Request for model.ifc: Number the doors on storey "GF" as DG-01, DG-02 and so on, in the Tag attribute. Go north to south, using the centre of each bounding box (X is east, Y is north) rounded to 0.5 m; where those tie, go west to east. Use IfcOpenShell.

First a look at what the model holds.

```python
import ifcopenshell
import ifcopenshell.util.element
import ifcopenshell.util.placement

model = ifcopenshell.open("model.ifc")
print(model.schema)
storey = next(s for s in model.by_type("IfcBuildingStorey") if s.Name == "GF")
doors = [e for e in ifcopenshell.util.element.get_decomposition(storey) if e.is_a("IfcDoor")]
for e in sorted(doors, key=lambda e: e.id()):
    origin = ifcopenshell.util.placement.get_local_placement(e.ObjectPlacement)[:3, 3]
    print(e.id(), e.Tag, e.Name, origin.round(2) + 0.0, sep=" | ")
```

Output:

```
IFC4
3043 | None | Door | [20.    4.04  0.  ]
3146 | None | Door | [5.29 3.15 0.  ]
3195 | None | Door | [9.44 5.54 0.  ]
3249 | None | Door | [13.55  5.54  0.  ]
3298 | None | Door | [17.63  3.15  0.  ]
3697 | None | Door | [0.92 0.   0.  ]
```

```python
import ifcopenshell
import ifcopenshell.geom
import ifcopenshell.util.element
import ifcopenshell.util.shape

model = ifcopenshell.open("model.ifc")
settings = ifcopenshell.geom.settings()
settings.set("use-world-coords", True)


def centre(element):
    shape = ifcopenshell.geom.create_shape(settings, element)
    return ifcopenshell.util.shape.get_bbox_centroid(shape.geometry)


storey = next(s for s in model.by_type("IfcBuildingStorey") if s.Name == "GF")
doors = [e for e in ifcopenshell.util.element.get_decomposition(storey) if e.is_a("IfcDoor")]

# Insertion points can sit at a corner or the storey origin, so sort by the geometry (in metres).
centres = {e: centre(e) for e in doors}
doors.sort(key=lambda e: (-round(centres[e][1] / 0.5), centres[e][0]))

for i, e in enumerate(doors, start=1):
    number = f"DG-{i:02d}"
    e.Tag = number
    print(e.id(), number)

model.write("model-out.ifc")
```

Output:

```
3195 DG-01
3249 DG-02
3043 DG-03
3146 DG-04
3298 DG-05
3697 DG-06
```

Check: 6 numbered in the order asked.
